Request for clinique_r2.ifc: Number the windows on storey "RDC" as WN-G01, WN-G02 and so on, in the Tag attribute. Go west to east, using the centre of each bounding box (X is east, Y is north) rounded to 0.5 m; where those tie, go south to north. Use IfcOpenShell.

First a look at what the model holds.

```python
import ifcopenshell
import ifcopenshell.util.element
import ifcopenshell.util.placement

model = ifcopenshell.open("clinique_r2.ifc")
print(model.schema)
storey = next(s for s in model.by_type("IfcBuildingStorey") if s.Name == "RDC")
windows = [e for e in ifcopenshell.util.element.get_decomposition(storey) if e.is_a("IfcWindow")]
for e in sorted(windows, key=lambda e: e.id()):
    origin = ifcopenshell.util.placement.get_local_placement(e.ObjectPlacement)[:3, 3]
    print(e.id(), e.Tag, e.Name, origin.round(2) + 0.0, sep=" | ")
```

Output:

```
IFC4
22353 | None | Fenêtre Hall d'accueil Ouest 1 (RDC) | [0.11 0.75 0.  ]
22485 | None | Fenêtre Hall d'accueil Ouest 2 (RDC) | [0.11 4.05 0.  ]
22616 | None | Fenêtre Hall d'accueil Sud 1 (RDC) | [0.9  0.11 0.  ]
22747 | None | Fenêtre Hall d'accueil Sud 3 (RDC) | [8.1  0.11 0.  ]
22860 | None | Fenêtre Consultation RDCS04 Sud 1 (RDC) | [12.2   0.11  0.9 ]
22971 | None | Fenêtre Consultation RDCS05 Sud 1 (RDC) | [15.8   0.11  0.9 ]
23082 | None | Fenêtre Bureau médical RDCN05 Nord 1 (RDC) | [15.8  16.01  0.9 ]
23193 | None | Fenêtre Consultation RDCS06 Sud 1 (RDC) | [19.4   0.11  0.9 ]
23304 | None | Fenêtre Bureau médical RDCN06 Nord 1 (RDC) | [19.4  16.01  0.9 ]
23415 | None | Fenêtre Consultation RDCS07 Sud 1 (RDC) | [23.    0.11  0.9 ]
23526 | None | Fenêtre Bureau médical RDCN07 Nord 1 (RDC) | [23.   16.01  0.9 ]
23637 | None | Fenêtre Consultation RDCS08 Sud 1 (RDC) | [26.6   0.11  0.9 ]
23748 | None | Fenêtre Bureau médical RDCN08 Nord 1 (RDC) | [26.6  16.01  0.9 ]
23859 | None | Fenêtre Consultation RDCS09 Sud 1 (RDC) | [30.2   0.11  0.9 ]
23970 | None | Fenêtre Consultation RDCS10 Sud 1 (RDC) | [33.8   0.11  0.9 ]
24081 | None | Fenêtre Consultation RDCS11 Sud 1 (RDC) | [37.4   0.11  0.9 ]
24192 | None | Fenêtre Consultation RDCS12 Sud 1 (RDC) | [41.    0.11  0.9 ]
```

```python
import ifcopenshell
import ifcopenshell.geom
import ifcopenshell.util.element
import ifcopenshell.util.shape

model = ifcopenshell.open("clinique_r2.ifc")
settings = ifcopenshell.geom.settings()
settings.set("use-world-coords", True)


def centre(element):
    shape = ifcopenshell.geom.create_shape(settings, element)
    return ifcopenshell.util.shape.get_bbox_centroid(shape.geometry)


storey = next(s for s in model.by_type("IfcBuildingStorey") if s.Name == "RDC")
windows = [e for e in ifcopenshell.util.element.get_decomposition(storey) if e.is_a("IfcWindow")]

# Insertion points can sit at a corner or the storey origin, so sort by the geometry (in metres).
centres = {e: centre(e) for e in windows}
windows.sort(key=lambda e: (round(centres[e][0] / 0.5), centres[e][1]))

for i, e in enumerate(windows, start=1):
    number = f"WN-G{i:02d}"
    e.Tag = number
    print(e.id(), number)

model.write("clinique_r2-out.ifc")
```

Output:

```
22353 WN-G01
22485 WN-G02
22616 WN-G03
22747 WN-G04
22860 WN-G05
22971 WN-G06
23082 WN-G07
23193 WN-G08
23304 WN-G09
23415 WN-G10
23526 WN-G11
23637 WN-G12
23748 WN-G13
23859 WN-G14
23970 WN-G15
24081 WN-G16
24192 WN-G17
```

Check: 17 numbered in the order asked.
